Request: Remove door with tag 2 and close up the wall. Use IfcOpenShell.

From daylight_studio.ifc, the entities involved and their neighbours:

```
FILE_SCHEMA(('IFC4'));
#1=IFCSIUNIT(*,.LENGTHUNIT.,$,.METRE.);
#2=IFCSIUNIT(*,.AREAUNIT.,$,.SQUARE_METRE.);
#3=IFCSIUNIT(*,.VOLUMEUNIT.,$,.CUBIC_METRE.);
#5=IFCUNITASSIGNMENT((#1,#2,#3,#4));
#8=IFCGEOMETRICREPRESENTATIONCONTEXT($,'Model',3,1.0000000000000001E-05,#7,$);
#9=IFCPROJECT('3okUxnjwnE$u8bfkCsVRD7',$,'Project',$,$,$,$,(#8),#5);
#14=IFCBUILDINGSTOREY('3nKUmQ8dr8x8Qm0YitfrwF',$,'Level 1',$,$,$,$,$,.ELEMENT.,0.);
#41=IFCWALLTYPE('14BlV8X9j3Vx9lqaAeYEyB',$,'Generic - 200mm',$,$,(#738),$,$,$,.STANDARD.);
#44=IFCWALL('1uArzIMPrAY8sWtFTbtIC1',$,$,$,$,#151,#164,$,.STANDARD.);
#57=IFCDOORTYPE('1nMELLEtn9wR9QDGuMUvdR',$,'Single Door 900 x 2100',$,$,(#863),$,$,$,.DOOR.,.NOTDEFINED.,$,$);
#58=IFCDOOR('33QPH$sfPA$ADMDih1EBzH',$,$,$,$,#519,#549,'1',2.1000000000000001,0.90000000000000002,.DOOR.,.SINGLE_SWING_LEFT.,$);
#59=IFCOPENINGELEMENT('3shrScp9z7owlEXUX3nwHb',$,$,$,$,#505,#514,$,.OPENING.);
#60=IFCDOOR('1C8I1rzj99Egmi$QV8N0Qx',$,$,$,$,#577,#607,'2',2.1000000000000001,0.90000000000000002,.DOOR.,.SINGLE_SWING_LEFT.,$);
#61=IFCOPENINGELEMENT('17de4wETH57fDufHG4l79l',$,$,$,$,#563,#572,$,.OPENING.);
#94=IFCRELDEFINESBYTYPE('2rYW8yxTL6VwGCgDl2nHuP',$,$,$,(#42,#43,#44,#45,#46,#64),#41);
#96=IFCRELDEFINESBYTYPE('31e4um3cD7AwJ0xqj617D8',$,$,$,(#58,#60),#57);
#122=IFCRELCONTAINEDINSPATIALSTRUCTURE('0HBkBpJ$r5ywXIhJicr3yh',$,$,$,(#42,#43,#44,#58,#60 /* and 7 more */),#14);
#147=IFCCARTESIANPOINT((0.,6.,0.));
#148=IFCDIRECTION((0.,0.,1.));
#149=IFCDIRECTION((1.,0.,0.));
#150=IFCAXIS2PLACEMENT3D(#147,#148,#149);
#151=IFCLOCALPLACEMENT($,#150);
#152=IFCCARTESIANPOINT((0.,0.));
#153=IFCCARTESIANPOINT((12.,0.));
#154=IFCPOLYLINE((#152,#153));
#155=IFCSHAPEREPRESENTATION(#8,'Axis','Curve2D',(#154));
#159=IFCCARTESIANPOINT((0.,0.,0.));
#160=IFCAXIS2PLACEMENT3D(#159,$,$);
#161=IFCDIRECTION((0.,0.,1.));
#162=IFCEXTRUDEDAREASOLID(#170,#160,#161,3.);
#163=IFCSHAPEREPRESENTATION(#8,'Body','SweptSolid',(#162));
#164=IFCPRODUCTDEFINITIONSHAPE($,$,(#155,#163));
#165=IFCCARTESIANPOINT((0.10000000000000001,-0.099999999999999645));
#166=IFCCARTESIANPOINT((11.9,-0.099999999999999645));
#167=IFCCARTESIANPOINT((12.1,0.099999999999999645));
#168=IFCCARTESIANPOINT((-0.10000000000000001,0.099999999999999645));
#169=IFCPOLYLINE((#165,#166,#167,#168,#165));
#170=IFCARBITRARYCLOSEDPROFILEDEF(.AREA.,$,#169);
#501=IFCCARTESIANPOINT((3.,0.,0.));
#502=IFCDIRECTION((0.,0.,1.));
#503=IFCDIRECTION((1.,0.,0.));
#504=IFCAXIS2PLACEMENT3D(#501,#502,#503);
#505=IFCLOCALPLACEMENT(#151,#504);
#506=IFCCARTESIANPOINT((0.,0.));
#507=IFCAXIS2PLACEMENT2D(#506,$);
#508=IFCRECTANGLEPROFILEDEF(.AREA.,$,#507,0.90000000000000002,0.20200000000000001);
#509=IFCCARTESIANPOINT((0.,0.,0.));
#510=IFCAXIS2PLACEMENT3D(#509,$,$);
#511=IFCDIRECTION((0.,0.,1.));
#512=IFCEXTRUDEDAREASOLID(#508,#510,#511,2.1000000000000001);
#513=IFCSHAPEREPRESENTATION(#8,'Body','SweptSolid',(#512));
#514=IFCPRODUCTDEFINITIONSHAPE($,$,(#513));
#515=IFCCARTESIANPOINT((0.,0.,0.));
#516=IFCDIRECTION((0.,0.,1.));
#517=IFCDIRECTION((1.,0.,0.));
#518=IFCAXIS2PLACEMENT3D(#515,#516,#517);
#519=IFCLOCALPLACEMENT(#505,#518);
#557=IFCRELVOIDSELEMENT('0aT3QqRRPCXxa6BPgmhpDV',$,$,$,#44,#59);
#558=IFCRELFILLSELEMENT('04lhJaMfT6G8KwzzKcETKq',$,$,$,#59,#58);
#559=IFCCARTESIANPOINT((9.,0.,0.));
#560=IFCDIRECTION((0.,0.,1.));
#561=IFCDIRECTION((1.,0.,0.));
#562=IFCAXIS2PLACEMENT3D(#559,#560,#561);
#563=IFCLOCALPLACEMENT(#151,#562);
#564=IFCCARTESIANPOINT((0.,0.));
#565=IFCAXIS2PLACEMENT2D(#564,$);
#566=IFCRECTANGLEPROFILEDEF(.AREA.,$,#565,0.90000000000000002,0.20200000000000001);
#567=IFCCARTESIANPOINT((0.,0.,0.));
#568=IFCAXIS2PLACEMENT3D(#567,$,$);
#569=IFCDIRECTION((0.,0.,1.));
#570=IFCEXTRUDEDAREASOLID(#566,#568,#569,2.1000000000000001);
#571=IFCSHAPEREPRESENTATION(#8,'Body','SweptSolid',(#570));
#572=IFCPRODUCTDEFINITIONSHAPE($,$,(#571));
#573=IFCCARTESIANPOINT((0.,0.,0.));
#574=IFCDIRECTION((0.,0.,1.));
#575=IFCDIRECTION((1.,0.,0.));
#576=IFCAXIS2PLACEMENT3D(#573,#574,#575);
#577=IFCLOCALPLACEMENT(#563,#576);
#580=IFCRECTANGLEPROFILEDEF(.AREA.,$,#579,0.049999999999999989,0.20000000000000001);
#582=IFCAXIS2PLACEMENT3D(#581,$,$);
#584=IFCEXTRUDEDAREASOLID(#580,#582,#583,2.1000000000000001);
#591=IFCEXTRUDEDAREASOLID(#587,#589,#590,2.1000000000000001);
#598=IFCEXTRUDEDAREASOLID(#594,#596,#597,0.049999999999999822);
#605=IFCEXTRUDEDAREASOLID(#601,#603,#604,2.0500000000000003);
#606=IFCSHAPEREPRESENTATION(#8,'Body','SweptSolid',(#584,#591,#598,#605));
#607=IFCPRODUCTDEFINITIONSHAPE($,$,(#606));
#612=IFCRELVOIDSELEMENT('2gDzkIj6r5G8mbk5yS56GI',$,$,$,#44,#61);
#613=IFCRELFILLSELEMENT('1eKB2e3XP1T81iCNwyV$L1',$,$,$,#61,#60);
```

```python
import ifcopenshell
import ifcopenshell.api.feature
import ifcopenshell.api.root
import ifcopenshell.geom
import ifcopenshell.util.shape

model = ifcopenshell.open("daylight_studio.ifc")
settings = ifcopenshell.geom.settings()


def volume(element):
    """Net volume in cubic metres, openings subtracted."""
    shape = ifcopenshell.geom.create_shape(settings, element)
    return ifcopenshell.util.shape.get_volume(shape.geometry)


door = model.by_guid("1C8I1rzj99Egmi$QV8N0Qx")
opening = door.FillsVoids[0].RelatingOpeningElement
wall = opening.VoidsElements[0].RelatingBuildingElement
before = volume(wall)

ifcopenshell.api.root.remove_product(model, product=door)
ifcopenshell.api.feature.remove_feature(model, feature=opening)

after = volume(wall)

print(f"wall volume {before:.3f} -> {after:.3f} m3")

model.write("daylight_studio_rev.ifc")
```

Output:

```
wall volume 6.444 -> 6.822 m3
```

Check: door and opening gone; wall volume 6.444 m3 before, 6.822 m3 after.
